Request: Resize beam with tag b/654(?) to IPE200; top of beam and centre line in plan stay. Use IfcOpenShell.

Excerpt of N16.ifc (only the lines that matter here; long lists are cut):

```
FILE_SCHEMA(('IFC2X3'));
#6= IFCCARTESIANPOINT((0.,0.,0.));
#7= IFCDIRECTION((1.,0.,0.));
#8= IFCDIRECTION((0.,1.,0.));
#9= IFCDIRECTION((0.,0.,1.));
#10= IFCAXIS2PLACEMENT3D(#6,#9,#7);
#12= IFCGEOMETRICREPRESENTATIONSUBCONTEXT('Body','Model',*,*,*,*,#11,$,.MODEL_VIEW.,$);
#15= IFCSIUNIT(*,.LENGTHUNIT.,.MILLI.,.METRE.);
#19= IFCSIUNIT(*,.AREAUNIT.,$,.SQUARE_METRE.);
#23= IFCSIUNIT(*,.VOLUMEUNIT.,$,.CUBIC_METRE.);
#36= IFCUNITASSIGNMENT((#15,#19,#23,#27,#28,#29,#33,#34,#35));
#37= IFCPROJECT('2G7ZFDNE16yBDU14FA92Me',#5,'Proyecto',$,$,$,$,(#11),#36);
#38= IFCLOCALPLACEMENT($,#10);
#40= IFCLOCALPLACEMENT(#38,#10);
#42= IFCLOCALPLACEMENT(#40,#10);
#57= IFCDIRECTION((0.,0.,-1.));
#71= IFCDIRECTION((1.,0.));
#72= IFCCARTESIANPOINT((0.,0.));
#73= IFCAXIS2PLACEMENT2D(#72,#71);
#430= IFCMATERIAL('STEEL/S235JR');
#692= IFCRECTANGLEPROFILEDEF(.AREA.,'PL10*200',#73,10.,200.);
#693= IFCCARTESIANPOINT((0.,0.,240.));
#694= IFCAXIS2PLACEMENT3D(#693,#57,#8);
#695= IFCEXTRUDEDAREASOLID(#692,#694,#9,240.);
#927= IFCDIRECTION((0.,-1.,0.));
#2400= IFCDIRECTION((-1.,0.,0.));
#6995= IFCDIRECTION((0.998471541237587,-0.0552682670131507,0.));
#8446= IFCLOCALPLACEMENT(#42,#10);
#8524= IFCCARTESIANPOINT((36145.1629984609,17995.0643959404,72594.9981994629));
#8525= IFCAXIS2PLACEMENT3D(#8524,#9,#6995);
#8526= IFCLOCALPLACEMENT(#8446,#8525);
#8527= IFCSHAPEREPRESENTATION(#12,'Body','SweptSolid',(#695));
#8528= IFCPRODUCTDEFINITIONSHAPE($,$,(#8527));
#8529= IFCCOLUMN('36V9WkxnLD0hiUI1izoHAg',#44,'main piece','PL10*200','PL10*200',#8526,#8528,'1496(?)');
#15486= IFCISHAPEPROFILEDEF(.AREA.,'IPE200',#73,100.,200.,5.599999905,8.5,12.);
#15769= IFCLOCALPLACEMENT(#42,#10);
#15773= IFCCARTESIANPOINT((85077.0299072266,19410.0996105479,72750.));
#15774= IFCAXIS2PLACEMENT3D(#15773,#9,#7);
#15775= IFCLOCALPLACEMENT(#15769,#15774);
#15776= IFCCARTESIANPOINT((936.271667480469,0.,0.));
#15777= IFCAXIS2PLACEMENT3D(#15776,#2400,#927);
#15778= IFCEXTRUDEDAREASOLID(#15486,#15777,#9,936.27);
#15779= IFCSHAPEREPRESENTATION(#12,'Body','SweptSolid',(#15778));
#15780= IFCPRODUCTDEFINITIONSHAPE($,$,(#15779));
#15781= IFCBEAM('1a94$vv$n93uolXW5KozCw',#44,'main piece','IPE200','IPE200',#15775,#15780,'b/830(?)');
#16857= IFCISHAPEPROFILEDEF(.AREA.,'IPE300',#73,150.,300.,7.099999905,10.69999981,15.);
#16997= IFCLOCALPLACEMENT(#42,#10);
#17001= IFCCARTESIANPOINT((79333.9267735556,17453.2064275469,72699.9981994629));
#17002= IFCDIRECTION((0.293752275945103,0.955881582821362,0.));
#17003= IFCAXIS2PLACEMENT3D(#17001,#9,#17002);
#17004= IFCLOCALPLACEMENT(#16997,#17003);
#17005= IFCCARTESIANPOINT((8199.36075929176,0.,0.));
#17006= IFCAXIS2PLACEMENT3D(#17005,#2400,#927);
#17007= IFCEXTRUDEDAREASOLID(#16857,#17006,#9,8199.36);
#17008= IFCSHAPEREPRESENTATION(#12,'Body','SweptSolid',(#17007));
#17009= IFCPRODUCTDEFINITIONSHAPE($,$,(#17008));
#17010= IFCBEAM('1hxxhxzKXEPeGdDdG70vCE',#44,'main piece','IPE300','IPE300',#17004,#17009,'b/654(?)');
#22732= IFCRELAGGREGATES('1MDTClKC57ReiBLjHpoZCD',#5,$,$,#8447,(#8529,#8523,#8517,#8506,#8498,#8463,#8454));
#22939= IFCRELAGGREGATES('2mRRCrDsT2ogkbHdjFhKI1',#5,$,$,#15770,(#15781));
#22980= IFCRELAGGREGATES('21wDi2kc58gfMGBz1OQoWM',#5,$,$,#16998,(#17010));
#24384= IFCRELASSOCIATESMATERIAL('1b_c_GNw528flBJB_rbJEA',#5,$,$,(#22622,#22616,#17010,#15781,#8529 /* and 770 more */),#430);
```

```python
import ifcopenshell
import ifcopenshell.util.element
import ifcopenshell.util.representation

model = ifcopenshell.open("N16.ifc")

member = model.by_guid("1hxxhxzKXEPeGdDdG70vCE")
source = next(p for p in model.by_type("IfcIShapeProfileDef") if p.ProfileName == "IPE200")

body = ifcopenshell.util.representation.get_representation(member, "Model", "Body")
solid = body.Items[0]
old_profile = solid.SweptArea

# Copy the section's sizes but keep this member's own profile position.
profile = ifcopenshell.util.element.copy(model, source)
# Profiles are centred, so shift by half the change in depth to hold the top.
shift = (old_profile.OverallDepth - profile.OverallDepth) / 2
x, y = old_profile.Position.Location.Coordinates
up = (0.0, 1.0)  # upwards, in the solid's own plane
location = model.createIfcCartesianPoint((x + up[0] * shift, y + up[1] * shift))
profile.Position = model.createIfcAxis2Placement2D(location, old_profile.Position.RefDirection)
solid.SweptArea = profile
if not model.get_total_inverses(old_profile):
    ifcopenshell.util.element.remove_deep2(model, old_profile)
member.Description = member.Description.replace("IPE300", "IPE200")
member.ObjectType = member.ObjectType.replace("IPE300", "IPE200")

print(solid.SweptArea)

model.write("N16_updated.ifc")
```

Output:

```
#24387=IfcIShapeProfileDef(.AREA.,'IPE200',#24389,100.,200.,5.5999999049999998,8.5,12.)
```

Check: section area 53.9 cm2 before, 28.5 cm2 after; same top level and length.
